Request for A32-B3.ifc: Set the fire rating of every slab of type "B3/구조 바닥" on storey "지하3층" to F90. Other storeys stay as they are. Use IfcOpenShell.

First a look at what the model holds.

```python
import ifcopenshell
import ifcopenshell.util.element

model = ifcopenshell.open("A32-B3.ifc")
print(model.schema)
storey = next(s for s in model.by_type("IfcBuildingStorey") if s.Name == "지하3층")
slabs = [e for e in ifcopenshell.util.element.get_decomposition(storey) if e.is_a("IfcSlab")]
seen = {}
for e in slabs:
    element_type = ifcopenshell.util.element.get_type(e)
    key = (element_type.Name if element_type != e and element_type else None, ifcopenshell.util.element.get_pset(e, "Pset_SlabCommon", "FireRating"))
    seen[key] = seen.get(key, 0) + 1
for (name, value), count in sorted(seen.items(), key=str):
    print(count, "x", name, "|", value)
```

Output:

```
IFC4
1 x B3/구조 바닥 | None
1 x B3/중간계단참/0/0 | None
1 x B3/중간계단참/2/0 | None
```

```python
import ifcopenshell
import ifcopenshell.api.pset
import ifcopenshell.util.element

model = ifcopenshell.open("A32-B3.ifc")

storey = next(s for s in model.by_type("IfcBuildingStorey") if s.Name == "지하3층")
slabs = [e for e in ifcopenshell.util.element.get_decomposition(storey) if e.is_a("IfcSlab")]

count = 0
for e in slabs:
    element_type = ifcopenshell.util.element.get_type(e)
    if element_type in (None, e) or element_type.Name != "B3/구조 바닥":
        continue
    # add_pset returns the element's existing set when there is one.
    pset = ifcopenshell.api.pset.add_pset(model, product=e, name="Pset_SlabCommon")
    ifcopenshell.api.pset.edit_pset(model, pset=pset, properties={"FireRating": "F90"})
    count += 1

print(count, "slabs updated")

model.write("A32-B3-out.ifc")
```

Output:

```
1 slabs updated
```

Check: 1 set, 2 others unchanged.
